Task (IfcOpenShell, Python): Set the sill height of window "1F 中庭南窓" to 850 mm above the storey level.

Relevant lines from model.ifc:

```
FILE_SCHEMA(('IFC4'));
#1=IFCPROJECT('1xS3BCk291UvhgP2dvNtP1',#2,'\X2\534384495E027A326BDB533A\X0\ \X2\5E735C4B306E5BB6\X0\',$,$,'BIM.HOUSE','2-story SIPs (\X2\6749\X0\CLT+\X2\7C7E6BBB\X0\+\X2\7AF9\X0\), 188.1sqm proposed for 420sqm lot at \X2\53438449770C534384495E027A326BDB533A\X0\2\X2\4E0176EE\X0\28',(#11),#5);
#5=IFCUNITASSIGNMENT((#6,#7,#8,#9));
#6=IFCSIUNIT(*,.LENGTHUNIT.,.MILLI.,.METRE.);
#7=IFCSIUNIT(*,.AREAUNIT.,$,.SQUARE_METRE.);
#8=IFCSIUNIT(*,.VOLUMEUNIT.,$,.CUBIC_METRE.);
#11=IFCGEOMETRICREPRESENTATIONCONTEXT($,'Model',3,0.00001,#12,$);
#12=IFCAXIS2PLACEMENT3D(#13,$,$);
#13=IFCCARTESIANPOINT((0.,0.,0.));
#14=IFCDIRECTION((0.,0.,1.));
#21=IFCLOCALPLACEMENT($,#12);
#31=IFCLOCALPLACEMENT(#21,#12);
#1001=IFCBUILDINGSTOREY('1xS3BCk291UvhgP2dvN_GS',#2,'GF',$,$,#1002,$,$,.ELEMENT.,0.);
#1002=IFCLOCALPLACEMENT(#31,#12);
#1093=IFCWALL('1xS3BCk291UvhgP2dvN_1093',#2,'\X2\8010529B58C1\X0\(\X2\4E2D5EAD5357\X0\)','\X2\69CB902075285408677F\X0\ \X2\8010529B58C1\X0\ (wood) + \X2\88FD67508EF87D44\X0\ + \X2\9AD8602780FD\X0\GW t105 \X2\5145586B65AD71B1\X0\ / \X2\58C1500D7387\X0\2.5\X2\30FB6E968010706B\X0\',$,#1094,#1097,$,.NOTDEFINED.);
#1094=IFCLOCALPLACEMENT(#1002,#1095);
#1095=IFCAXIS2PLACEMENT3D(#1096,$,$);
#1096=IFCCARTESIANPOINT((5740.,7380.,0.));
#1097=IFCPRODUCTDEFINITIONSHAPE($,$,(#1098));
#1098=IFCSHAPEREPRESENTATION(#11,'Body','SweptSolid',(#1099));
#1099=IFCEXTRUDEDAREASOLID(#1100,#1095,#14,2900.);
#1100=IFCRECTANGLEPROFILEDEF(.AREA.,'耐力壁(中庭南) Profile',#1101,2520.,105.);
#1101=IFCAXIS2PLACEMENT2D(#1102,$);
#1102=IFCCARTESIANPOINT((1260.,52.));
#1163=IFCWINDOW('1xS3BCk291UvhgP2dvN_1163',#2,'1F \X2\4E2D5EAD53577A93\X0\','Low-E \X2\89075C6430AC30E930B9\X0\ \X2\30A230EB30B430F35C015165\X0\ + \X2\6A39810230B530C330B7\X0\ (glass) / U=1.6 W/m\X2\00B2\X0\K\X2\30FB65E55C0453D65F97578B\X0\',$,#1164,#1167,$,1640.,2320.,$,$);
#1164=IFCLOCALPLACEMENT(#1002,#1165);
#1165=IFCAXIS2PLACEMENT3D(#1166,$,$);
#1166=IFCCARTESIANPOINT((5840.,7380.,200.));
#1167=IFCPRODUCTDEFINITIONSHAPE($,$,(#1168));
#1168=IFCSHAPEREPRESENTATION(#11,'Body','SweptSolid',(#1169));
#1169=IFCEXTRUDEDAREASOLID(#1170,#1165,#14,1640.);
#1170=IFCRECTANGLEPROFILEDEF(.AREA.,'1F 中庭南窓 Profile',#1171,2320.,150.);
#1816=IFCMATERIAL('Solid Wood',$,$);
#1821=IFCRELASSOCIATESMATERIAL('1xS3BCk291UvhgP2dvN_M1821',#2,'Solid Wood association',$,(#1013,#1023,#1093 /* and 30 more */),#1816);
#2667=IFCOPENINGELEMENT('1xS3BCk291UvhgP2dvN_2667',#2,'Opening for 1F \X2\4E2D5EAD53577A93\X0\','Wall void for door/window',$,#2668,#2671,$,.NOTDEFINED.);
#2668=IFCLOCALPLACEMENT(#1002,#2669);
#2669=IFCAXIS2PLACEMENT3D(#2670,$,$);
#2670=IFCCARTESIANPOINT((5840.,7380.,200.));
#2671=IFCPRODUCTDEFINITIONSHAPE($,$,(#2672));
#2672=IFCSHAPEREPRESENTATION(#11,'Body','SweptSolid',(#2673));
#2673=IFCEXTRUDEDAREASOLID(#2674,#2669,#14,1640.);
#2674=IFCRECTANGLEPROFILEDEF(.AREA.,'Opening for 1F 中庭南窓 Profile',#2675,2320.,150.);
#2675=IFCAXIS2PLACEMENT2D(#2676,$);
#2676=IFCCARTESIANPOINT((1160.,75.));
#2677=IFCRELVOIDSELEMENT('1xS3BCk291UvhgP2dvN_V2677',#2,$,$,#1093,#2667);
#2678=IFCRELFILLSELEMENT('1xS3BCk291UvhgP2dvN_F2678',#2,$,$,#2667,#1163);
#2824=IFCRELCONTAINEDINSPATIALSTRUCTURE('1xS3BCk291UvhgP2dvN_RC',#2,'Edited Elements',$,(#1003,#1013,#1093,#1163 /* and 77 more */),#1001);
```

```python
import numpy as np
import ifcopenshell
import ifcopenshell.api.geometry
import ifcopenshell.geom
import ifcopenshell.util.element
import ifcopenshell.util.placement
import ifcopenshell.util.shape
import ifcopenshell.util.unit

model = ifcopenshell.open("model.ifc")
unit_scale = ifcopenshell.util.unit.calculate_unit_scale(model)

window = model.by_guid("1xS3BCk291UvhgP2dvN_1163")
opening = window.FillsVoids[0].RelatingOpeningElement
storey = ifcopenshell.util.element.get_container(window, ifc_class="IfcBuildingStorey")
level = ifcopenshell.util.placement.get_local_placement(storey.ObjectPlacement)[2, 3]

# The opening's origin need not be at the sill, so measure its lowest point.
shape = ifcopenshell.geom.create_shape(ifcopenshell.geom.settings(), opening)
bottom = ifcopenshell.util.shape.get_shape_bottom_elevation(shape, shape.geometry) / unit_scale
dz = level + 0.85 / unit_scale - bottom

shift = np.array([0.0, 0.0, dz])
# The window is not placed relative to its opening, so move both.
for product in (opening, window):
    matrix = ifcopenshell.util.placement.get_local_placement(product.ObjectPlacement)
    matrix[:3, 3] += shift
    ifcopenshell.api.geometry.edit_object_placement(model, product=product, matrix=matrix, is_si=False)

print(f"moved by {dz * unit_scale:+.3f} m")

model.write("model_updated.ifc")
```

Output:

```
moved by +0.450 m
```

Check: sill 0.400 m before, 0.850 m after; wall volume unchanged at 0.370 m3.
